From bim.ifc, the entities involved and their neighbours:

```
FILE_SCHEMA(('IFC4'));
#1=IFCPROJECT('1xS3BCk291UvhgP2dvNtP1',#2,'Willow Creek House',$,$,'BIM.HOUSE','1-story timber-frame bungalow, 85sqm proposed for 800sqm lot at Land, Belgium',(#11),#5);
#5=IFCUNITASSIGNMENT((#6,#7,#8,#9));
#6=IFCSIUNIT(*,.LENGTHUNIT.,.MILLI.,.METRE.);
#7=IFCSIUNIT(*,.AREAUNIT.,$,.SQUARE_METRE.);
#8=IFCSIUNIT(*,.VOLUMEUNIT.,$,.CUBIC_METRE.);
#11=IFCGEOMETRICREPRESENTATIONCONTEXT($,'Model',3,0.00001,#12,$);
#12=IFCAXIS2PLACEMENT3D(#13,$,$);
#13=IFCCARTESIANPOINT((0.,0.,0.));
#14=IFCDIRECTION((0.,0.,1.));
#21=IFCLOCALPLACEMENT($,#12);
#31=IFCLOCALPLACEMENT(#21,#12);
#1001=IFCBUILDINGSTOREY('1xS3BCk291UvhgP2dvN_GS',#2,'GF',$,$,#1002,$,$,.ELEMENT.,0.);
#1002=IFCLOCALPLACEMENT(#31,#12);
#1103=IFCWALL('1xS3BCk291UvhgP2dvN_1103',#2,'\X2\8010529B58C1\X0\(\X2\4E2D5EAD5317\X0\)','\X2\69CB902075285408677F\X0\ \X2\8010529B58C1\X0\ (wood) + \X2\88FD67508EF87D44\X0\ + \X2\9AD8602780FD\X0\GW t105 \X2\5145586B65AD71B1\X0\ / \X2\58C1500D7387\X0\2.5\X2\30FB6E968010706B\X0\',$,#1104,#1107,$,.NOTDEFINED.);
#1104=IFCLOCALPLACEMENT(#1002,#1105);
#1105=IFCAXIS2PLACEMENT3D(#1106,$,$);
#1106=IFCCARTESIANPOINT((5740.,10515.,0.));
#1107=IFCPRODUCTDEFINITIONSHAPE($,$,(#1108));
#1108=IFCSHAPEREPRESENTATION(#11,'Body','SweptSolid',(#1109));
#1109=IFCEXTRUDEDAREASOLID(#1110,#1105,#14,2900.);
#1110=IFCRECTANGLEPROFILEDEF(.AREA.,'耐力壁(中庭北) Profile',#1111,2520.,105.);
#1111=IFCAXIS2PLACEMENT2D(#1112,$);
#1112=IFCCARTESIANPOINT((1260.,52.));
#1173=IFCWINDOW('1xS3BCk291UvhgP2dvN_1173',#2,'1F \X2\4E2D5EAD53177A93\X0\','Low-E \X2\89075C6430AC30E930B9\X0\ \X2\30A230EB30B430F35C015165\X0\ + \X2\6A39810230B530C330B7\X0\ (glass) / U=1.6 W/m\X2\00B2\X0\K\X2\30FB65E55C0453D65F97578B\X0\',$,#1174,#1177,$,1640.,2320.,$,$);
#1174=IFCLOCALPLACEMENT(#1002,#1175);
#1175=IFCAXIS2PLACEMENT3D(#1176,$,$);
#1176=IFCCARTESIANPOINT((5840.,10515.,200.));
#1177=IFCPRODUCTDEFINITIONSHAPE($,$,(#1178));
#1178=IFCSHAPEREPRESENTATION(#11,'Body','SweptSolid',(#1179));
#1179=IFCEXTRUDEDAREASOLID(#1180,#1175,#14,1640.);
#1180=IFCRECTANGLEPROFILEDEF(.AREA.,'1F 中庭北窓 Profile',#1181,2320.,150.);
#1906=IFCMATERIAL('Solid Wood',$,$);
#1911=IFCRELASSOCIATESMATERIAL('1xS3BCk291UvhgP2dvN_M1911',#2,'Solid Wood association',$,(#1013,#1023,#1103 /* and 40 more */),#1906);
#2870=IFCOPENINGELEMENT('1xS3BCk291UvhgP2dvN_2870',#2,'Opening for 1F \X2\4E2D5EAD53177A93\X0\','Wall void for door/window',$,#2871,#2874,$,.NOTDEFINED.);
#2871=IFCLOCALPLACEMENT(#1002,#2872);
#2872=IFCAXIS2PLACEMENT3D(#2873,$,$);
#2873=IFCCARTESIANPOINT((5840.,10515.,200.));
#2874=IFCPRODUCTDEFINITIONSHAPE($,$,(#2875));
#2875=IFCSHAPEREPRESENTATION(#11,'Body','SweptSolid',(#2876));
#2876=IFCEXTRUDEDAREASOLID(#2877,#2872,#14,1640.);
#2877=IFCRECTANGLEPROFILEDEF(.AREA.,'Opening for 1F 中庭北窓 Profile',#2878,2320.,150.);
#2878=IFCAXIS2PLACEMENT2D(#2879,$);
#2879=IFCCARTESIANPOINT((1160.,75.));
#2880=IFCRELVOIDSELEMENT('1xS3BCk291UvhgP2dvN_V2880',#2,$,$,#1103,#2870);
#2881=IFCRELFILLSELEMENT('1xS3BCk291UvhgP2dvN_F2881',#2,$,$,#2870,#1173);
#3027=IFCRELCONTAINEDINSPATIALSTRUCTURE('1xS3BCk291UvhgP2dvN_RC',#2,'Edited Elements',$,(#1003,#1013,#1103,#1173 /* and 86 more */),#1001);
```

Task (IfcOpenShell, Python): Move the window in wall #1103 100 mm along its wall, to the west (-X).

```python
import ifcopenshell
import ifcopenshell.api.geometry
import ifcopenshell.util.placement
import ifcopenshell.util.unit

model = ifcopenshell.open("bim.ifc")
unit_scale = ifcopenshell.util.unit.calculate_unit_scale(model)

window = model.by_id(1173)
opening = window.FillsVoids[0].RelatingOpeningElement
wall = opening.VoidsElements[0].RelatingBuildingElement

wall_matrix = ifcopenshell.util.placement.get_local_placement(wall.ObjectPlacement)
shift = wall_matrix[:3, 0] * -0.1 / unit_scale
before = ifcopenshell.util.placement.get_local_placement(window.ObjectPlacement)[:3, 3].copy()

# The window is not placed relative to its opening, so move both.
for product in (opening, window):
    matrix = ifcopenshell.util.placement.get_local_placement(product.ObjectPlacement)
    matrix[:3, 3] += shift
    ifcopenshell.api.geometry.edit_object_placement(model, product=product, matrix=matrix, is_si=False)

after = ifcopenshell.util.placement.get_local_placement(window.ObjectPlacement)[:3, 3]
print("window moved by", (after - before).round(3) + 0.0)

model.write("bim_edited.ifc")
```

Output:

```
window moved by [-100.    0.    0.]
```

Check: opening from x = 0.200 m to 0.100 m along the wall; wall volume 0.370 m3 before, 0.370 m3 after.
